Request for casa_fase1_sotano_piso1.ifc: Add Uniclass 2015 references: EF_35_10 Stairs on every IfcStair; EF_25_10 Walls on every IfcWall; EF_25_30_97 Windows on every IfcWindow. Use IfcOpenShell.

First a look at what the model holds.

```python
import ifcopenshell

model = ifcopenshell.open("casa_fase1_sotano_piso1.ifc")
print(model.schema)
print("classifications:", [c.Name for c in model.by_type("IfcClassification")])
for ifc_class in ("IfcDoor", "IfcRoof", "IfcStair", "IfcWall", "IfcWindow"):
    print(ifc_class, len(model.by_type(ifc_class)))
```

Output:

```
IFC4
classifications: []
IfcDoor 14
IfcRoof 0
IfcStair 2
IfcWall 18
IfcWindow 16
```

```python
import ifcopenshell
import ifcopenshell.api.classification

model = ifcopenshell.open("casa_fase1_sotano_piso1.ifc")

system = ifcopenshell.api.classification.add_classification(model, classification="Uniclass 2015")

codes = {
    "IfcStair": ("EF_35_10", "Stairs"),
    "IfcWall": ("EF_25_10", "Walls"),
    "IfcWindow": ("EF_25_30_97", "Windows"),
}
for ifc_class, (code, name) in codes.items():
    products = model.by_type(ifc_class)
    ifcopenshell.api.classification.add_reference(
        model, products=products, classification=system, identification=code, name=name
    )
    print(code, len(products))

model.write("casa_fase1_sotano_piso1_v2.ifc")
```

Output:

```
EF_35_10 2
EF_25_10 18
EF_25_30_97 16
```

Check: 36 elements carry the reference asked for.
